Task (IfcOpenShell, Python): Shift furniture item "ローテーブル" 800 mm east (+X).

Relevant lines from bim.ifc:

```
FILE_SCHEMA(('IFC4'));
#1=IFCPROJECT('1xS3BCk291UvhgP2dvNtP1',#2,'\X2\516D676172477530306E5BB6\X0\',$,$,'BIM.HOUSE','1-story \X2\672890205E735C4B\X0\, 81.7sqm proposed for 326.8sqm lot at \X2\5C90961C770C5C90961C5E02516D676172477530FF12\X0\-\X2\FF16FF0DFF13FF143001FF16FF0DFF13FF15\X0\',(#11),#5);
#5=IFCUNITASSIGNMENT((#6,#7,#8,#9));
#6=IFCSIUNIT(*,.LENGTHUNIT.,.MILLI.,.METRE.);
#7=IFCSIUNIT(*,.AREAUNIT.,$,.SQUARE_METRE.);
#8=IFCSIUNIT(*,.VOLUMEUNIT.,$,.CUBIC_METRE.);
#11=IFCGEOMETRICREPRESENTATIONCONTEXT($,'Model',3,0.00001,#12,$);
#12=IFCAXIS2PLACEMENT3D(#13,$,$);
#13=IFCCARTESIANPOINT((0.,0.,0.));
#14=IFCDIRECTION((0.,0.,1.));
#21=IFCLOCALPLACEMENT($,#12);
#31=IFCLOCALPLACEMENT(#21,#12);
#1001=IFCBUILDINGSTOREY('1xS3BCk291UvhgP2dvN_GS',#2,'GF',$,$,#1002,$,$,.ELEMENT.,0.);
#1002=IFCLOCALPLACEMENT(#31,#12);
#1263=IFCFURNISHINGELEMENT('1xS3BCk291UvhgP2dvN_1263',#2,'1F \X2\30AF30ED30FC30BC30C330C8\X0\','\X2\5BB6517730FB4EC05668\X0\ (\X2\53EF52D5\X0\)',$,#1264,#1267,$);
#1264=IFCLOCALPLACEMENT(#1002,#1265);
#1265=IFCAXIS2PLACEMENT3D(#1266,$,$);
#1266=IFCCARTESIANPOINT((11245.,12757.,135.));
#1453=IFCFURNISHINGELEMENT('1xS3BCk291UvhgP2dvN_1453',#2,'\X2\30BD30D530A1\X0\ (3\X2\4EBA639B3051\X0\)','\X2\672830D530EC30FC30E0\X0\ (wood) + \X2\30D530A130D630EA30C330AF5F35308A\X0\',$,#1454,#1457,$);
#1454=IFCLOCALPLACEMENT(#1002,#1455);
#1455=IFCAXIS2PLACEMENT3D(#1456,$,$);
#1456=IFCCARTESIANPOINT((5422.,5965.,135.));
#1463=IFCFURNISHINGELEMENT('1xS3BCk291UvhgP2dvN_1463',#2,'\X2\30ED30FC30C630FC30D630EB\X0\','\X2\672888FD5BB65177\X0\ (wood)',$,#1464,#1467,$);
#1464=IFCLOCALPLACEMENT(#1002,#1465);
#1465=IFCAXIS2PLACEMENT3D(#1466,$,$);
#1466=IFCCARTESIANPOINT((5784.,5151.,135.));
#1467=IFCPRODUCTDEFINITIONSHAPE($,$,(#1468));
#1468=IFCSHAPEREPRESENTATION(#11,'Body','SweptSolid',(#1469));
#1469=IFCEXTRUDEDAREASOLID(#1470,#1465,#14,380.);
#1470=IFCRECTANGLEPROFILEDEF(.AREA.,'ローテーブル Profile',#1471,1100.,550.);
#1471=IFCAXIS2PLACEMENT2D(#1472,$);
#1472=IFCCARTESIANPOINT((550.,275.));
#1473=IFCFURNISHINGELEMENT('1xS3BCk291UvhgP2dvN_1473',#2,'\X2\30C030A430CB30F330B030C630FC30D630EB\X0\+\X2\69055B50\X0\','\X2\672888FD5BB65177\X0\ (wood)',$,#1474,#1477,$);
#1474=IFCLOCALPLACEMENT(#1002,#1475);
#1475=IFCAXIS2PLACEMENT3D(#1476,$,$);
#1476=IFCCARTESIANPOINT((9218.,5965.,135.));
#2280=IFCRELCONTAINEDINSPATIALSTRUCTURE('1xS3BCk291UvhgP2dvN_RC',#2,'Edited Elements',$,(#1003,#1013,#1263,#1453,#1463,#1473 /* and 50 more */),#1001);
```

```python
import ifcopenshell
import ifcopenshell.api.geometry
import ifcopenshell.util.placement
import ifcopenshell.util.unit

model = ifcopenshell.open("bim.ifc")
unit_scale = ifcopenshell.util.unit.calculate_unit_scale(model)

item = model.by_guid("1xS3BCk291UvhgP2dvN_1463")
matrix = ifcopenshell.util.placement.get_local_placement(item.ObjectPlacement)
matrix[0, 3] += 0.8 / unit_scale
ifcopenshell.api.geometry.edit_object_placement(model, product=item, matrix=matrix, is_si=False)

print(ifcopenshell.util.placement.get_local_placement(item.ObjectPlacement).round(3) + 0.0)

model.write("bim_updated.ifc")
```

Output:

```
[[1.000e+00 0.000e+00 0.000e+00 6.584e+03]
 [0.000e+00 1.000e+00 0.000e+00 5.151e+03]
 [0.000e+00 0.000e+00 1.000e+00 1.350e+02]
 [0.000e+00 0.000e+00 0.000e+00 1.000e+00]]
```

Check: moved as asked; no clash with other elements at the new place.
